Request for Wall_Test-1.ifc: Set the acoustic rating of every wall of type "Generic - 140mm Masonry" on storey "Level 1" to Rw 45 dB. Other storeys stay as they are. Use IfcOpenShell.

First a look at what the model holds.

```python
import ifcopenshell
import ifcopenshell.util.element

model = ifcopenshell.open("Wall_Test-1.ifc")
print(model.schema)
storey = next(s for s in model.by_type("IfcBuildingStorey") if s.Name == "Level 1")
walls = [e for e in ifcopenshell.util.element.get_decomposition(storey) if e.is_a("IfcWall")]
seen = {}
for e in walls:
    element_type = ifcopenshell.util.element.get_type(e)
    key = (element_type.Name if element_type != e and element_type else None, ifcopenshell.util.element.get_pset(e, "Pset_WallCommon", "AcousticRating"))
    seen[key] = seen.get(key, 0) + 1
for (name, value), count in sorted(seen.items(), key=str):
    print(count, "x", name, "|", value)
```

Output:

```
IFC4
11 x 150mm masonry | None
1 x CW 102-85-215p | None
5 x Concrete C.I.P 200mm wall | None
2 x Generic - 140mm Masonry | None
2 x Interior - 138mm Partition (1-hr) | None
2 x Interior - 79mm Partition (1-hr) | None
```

```python
import ifcopenshell
import ifcopenshell.api.pset
import ifcopenshell.util.element

model = ifcopenshell.open("Wall_Test-1.ifc")

storey = next(s for s in model.by_type("IfcBuildingStorey") if s.Name == "Level 1")
walls = [e for e in ifcopenshell.util.element.get_decomposition(storey) if e.is_a("IfcWall")]

count = 0
for e in walls:
    element_type = ifcopenshell.util.element.get_type(e)
    if element_type in (None, e) or element_type.Name != "Generic - 140mm Masonry":
        continue
    # add_pset returns the element's existing set when there is one.
    pset = ifcopenshell.api.pset.add_pset(model, product=e, name="Pset_WallCommon")
    ifcopenshell.api.pset.edit_pset(model, pset=pset, properties={"AcousticRating": "Rw 45 dB"})
    count += 1

print(count, "walls updated")

model.write("Wall_Test-1_edited.ifc")
```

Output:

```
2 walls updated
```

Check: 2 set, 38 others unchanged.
